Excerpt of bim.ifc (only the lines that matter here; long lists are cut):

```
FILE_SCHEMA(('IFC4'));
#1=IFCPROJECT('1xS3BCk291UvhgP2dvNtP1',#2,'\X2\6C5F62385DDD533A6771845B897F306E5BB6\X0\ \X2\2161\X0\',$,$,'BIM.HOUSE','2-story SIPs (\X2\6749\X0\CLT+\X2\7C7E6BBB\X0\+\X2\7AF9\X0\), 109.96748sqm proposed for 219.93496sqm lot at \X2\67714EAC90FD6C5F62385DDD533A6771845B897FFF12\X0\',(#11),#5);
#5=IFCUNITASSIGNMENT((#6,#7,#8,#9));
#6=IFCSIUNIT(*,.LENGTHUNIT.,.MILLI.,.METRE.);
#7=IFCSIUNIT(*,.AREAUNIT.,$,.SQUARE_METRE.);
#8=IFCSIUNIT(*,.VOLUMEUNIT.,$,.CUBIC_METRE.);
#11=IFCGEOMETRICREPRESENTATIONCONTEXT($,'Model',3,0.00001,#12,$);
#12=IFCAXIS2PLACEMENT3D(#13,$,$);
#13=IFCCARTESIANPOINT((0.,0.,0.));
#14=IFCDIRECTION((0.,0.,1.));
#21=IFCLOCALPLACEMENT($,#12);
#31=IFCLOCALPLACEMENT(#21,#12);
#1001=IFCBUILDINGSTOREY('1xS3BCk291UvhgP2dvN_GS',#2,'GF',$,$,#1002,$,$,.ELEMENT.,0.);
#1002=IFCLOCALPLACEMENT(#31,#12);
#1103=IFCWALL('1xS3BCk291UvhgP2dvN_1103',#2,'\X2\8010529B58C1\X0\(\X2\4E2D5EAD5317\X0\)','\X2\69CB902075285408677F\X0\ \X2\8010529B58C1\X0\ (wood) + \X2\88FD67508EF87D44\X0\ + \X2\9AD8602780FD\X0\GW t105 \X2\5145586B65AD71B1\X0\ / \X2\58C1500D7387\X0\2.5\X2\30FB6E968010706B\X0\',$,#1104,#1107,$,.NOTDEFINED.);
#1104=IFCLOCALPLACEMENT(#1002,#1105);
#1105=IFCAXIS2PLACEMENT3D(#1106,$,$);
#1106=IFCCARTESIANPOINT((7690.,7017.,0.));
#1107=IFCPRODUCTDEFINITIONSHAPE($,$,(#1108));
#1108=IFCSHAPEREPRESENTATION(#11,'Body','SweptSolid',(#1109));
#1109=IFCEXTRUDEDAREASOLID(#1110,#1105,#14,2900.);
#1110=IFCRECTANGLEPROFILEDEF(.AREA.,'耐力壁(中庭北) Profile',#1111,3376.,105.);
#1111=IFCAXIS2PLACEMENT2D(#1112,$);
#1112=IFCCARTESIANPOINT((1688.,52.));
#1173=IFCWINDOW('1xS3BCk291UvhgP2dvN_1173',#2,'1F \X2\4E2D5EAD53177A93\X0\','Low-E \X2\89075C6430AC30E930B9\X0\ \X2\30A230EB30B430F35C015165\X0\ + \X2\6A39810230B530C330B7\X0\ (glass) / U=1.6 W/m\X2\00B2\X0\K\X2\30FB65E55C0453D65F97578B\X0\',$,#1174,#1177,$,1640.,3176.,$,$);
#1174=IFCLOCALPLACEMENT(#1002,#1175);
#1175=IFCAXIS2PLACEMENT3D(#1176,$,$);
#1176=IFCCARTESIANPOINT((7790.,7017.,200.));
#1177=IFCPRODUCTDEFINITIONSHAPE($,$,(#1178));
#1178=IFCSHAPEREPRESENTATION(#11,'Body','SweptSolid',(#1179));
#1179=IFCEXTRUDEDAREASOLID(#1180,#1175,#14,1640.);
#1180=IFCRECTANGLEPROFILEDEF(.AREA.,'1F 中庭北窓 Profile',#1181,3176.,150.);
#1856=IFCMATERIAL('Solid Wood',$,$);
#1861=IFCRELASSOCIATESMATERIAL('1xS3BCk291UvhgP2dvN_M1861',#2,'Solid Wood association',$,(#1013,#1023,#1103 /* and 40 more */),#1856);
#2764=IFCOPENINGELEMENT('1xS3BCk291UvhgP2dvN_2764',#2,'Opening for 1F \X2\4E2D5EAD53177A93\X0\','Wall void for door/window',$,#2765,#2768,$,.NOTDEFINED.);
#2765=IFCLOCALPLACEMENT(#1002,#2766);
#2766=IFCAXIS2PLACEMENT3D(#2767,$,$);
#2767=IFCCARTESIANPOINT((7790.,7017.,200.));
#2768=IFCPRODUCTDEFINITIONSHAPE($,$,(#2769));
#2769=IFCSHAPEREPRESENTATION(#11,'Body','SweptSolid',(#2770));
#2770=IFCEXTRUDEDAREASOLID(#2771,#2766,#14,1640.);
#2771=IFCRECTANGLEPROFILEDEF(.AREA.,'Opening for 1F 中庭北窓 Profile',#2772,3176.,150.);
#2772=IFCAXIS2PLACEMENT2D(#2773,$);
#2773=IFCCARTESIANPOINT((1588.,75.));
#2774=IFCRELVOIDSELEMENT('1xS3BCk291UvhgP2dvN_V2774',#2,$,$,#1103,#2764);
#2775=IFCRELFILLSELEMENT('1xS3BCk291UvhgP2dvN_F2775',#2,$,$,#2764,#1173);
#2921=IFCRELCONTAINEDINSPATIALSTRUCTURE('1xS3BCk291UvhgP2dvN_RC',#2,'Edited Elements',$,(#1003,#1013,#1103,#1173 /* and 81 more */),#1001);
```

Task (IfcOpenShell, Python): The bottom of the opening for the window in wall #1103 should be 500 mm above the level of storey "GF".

```python
import numpy as np
import ifcopenshell
import ifcopenshell.api.geometry
import ifcopenshell.geom
import ifcopenshell.util.element
import ifcopenshell.util.placement
import ifcopenshell.util.shape
import ifcopenshell.util.unit

model = ifcopenshell.open("bim.ifc")
unit_scale = ifcopenshell.util.unit.calculate_unit_scale(model)

window = model.by_guid("1xS3BCk291UvhgP2dvN_1173")
opening = window.FillsVoids[0].RelatingOpeningElement
storey = ifcopenshell.util.element.get_container(window, ifc_class="IfcBuildingStorey")
level = ifcopenshell.util.placement.get_local_placement(storey.ObjectPlacement)[2, 3]

# The opening's origin need not be at the sill, so measure its lowest point.
shape = ifcopenshell.geom.create_shape(ifcopenshell.geom.settings(), opening)
bottom = ifcopenshell.util.shape.get_shape_bottom_elevation(shape, shape.geometry) / unit_scale
dz = level + 0.5 / unit_scale - bottom

shift = np.array([0.0, 0.0, dz])
# The window is not placed relative to its opening, so move both.
for product in (opening, window):
    matrix = ifcopenshell.util.placement.get_local_placement(product.ObjectPlacement)
    matrix[:3, 3] += shift
    ifcopenshell.api.geometry.edit_object_placement(model, product=product, matrix=matrix, is_si=False)

print(f"moved by {dz * unit_scale:+.3f} m")

model.write("bim-out.ifc")
```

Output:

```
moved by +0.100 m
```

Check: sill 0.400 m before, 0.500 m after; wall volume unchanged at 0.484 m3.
